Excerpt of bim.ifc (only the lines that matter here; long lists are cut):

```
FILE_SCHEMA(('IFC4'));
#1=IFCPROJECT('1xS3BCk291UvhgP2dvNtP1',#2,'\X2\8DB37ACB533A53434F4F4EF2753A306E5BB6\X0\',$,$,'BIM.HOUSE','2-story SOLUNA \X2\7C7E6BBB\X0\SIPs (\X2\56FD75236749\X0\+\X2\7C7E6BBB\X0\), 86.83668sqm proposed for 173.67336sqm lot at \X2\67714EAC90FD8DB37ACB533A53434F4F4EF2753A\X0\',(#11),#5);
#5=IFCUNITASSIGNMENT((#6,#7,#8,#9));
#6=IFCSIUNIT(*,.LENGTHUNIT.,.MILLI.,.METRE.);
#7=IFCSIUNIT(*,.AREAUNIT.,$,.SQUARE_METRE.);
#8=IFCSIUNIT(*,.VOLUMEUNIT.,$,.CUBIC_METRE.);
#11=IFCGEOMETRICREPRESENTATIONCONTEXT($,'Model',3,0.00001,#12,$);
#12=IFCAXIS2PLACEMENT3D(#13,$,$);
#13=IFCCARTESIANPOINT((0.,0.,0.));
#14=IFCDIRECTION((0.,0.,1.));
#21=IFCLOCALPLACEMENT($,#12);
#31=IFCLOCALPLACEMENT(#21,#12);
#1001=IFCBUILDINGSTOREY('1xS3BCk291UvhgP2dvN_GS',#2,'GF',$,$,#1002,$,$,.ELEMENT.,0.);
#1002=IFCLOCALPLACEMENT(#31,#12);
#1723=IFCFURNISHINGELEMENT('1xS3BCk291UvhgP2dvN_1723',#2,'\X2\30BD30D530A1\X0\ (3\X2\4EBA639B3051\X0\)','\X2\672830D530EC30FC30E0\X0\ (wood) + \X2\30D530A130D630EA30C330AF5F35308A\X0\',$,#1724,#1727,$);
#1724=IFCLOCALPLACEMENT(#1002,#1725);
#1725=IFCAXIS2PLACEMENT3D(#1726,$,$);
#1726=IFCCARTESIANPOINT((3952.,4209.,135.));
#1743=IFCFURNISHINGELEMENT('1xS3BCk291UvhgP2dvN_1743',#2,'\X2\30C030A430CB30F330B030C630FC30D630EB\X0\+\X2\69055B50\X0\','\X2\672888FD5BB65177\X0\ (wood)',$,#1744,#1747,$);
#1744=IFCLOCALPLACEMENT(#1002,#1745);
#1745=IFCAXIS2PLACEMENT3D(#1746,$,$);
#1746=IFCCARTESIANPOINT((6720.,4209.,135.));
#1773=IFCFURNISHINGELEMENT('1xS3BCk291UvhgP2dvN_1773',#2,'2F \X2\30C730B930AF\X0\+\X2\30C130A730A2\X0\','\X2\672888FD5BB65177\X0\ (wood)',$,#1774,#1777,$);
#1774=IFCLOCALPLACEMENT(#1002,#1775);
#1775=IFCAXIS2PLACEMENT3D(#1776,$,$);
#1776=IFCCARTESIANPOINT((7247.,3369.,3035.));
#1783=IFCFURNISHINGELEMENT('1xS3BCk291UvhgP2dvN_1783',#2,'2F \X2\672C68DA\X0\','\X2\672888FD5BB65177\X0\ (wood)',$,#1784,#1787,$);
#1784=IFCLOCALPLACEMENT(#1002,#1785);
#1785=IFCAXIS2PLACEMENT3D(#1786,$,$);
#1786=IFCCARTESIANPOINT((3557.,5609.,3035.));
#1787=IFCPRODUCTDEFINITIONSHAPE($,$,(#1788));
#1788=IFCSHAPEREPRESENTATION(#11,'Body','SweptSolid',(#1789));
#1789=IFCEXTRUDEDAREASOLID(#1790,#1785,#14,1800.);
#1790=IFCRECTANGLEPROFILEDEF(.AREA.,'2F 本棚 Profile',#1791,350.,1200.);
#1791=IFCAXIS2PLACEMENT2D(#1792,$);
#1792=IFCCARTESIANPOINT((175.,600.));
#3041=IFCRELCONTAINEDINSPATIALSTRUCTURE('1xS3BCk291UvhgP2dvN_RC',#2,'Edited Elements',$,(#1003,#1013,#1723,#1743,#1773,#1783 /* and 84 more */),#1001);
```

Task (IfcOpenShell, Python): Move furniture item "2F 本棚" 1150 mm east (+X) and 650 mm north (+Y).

```python
import ifcopenshell
import ifcopenshell.api.geometry
import ifcopenshell.util.placement

model = ifcopenshell.open("bim.ifc")

item = model.by_id(1783)
matrix = ifcopenshell.util.placement.get_local_placement(item.ObjectPlacement)
matrix[0, 3] += 1150.0
matrix[1, 3] += 650.0
ifcopenshell.api.geometry.edit_object_placement(model, product=item, matrix=matrix, is_si=False)

print(ifcopenshell.util.placement.get_local_placement(item.ObjectPlacement).round(3) + 0.0)

model.write("bim-out.ifc")
```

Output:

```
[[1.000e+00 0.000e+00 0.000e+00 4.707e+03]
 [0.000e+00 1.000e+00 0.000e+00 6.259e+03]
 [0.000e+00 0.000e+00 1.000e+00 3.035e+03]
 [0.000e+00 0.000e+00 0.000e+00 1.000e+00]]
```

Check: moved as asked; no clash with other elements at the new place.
